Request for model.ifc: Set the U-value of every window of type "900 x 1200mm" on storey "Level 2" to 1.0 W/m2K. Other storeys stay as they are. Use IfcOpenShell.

First a look at what the model holds.

```python
import ifcopenshell
import ifcopenshell.util.element

model = ifcopenshell.open("model.ifc")
print(model.schema)
storey = next(s for s in model.by_type("IfcBuildingStorey") if s.Name == "Level 2")
windows = [e for e in ifcopenshell.util.element.get_decomposition(storey) if e.is_a("IfcWindow")]
seen = {}
for e in windows:
    element_type = ifcopenshell.util.element.get_type(e)
    key = (element_type.Name if element_type != e and element_type else None, ifcopenshell.util.element.get_pset(e, "Pset_WindowCommon", "ThermalTransmittance"))
    seen[key] = seen.get(key, 0) + 1
for (name, value), count in sorted(seen.items(), key=str):
    print(count, "x", name, "|", value)
```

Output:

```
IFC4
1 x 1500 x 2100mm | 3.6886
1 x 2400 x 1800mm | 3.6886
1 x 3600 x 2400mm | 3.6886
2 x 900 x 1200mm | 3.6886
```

```python
import ifcopenshell
import ifcopenshell.api.pset
import ifcopenshell.util.element

model = ifcopenshell.open("model.ifc")

storey = next(s for s in model.by_type("IfcBuildingStorey") if s.Name == "Level 2")
windows = [e for e in ifcopenshell.util.element.get_decomposition(storey) if e.is_a("IfcWindow")]

count = 0
for e in windows:
    element_type = ifcopenshell.util.element.get_type(e)
    if element_type in (None, e) or element_type.Name != "900 x 1200mm":
        continue
    # add_pset returns the element's existing set when there is one.
    pset = ifcopenshell.api.pset.add_pset(model, product=e, name="Pset_WindowCommon")
    ifcopenshell.api.pset.edit_pset(model, pset=pset, properties={"ThermalTransmittance": 1.0})
    count += 1

print(count, "windows updated")

model.write("model_rev.ifc")
```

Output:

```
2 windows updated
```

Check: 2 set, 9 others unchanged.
